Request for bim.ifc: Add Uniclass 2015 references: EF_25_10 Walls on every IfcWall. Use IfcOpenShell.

First a look at what the model holds.

```python
import ifcopenshell

model = ifcopenshell.open("bim.ifc")
print(model.schema)
print("classifications:", [c.Name for c in model.by_type("IfcClassification")])
for ifc_class in ("IfcDoor", "IfcRoof", "IfcStair", "IfcWall", "IfcWindow"):
    print(ifc_class, len(model.by_type(ifc_class)))
```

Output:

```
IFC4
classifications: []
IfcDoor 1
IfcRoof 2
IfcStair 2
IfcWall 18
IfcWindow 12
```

```python
import ifcopenshell
import ifcopenshell.api.classification

model = ifcopenshell.open("bim.ifc")

system = ifcopenshell.api.classification.add_classification(model, classification="Uniclass 2015")

codes = {
    "IfcWall": ("EF_25_10", "Walls"),
}
for ifc_class, (code, name) in codes.items():
    products = model.by_type(ifc_class)
    ifcopenshell.api.classification.add_reference(
        model, products=products, classification=system, identification=code, name=name
    )
    print(code, len(products))

model.write("bim_rev.ifc")
```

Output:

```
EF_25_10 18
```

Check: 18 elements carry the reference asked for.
